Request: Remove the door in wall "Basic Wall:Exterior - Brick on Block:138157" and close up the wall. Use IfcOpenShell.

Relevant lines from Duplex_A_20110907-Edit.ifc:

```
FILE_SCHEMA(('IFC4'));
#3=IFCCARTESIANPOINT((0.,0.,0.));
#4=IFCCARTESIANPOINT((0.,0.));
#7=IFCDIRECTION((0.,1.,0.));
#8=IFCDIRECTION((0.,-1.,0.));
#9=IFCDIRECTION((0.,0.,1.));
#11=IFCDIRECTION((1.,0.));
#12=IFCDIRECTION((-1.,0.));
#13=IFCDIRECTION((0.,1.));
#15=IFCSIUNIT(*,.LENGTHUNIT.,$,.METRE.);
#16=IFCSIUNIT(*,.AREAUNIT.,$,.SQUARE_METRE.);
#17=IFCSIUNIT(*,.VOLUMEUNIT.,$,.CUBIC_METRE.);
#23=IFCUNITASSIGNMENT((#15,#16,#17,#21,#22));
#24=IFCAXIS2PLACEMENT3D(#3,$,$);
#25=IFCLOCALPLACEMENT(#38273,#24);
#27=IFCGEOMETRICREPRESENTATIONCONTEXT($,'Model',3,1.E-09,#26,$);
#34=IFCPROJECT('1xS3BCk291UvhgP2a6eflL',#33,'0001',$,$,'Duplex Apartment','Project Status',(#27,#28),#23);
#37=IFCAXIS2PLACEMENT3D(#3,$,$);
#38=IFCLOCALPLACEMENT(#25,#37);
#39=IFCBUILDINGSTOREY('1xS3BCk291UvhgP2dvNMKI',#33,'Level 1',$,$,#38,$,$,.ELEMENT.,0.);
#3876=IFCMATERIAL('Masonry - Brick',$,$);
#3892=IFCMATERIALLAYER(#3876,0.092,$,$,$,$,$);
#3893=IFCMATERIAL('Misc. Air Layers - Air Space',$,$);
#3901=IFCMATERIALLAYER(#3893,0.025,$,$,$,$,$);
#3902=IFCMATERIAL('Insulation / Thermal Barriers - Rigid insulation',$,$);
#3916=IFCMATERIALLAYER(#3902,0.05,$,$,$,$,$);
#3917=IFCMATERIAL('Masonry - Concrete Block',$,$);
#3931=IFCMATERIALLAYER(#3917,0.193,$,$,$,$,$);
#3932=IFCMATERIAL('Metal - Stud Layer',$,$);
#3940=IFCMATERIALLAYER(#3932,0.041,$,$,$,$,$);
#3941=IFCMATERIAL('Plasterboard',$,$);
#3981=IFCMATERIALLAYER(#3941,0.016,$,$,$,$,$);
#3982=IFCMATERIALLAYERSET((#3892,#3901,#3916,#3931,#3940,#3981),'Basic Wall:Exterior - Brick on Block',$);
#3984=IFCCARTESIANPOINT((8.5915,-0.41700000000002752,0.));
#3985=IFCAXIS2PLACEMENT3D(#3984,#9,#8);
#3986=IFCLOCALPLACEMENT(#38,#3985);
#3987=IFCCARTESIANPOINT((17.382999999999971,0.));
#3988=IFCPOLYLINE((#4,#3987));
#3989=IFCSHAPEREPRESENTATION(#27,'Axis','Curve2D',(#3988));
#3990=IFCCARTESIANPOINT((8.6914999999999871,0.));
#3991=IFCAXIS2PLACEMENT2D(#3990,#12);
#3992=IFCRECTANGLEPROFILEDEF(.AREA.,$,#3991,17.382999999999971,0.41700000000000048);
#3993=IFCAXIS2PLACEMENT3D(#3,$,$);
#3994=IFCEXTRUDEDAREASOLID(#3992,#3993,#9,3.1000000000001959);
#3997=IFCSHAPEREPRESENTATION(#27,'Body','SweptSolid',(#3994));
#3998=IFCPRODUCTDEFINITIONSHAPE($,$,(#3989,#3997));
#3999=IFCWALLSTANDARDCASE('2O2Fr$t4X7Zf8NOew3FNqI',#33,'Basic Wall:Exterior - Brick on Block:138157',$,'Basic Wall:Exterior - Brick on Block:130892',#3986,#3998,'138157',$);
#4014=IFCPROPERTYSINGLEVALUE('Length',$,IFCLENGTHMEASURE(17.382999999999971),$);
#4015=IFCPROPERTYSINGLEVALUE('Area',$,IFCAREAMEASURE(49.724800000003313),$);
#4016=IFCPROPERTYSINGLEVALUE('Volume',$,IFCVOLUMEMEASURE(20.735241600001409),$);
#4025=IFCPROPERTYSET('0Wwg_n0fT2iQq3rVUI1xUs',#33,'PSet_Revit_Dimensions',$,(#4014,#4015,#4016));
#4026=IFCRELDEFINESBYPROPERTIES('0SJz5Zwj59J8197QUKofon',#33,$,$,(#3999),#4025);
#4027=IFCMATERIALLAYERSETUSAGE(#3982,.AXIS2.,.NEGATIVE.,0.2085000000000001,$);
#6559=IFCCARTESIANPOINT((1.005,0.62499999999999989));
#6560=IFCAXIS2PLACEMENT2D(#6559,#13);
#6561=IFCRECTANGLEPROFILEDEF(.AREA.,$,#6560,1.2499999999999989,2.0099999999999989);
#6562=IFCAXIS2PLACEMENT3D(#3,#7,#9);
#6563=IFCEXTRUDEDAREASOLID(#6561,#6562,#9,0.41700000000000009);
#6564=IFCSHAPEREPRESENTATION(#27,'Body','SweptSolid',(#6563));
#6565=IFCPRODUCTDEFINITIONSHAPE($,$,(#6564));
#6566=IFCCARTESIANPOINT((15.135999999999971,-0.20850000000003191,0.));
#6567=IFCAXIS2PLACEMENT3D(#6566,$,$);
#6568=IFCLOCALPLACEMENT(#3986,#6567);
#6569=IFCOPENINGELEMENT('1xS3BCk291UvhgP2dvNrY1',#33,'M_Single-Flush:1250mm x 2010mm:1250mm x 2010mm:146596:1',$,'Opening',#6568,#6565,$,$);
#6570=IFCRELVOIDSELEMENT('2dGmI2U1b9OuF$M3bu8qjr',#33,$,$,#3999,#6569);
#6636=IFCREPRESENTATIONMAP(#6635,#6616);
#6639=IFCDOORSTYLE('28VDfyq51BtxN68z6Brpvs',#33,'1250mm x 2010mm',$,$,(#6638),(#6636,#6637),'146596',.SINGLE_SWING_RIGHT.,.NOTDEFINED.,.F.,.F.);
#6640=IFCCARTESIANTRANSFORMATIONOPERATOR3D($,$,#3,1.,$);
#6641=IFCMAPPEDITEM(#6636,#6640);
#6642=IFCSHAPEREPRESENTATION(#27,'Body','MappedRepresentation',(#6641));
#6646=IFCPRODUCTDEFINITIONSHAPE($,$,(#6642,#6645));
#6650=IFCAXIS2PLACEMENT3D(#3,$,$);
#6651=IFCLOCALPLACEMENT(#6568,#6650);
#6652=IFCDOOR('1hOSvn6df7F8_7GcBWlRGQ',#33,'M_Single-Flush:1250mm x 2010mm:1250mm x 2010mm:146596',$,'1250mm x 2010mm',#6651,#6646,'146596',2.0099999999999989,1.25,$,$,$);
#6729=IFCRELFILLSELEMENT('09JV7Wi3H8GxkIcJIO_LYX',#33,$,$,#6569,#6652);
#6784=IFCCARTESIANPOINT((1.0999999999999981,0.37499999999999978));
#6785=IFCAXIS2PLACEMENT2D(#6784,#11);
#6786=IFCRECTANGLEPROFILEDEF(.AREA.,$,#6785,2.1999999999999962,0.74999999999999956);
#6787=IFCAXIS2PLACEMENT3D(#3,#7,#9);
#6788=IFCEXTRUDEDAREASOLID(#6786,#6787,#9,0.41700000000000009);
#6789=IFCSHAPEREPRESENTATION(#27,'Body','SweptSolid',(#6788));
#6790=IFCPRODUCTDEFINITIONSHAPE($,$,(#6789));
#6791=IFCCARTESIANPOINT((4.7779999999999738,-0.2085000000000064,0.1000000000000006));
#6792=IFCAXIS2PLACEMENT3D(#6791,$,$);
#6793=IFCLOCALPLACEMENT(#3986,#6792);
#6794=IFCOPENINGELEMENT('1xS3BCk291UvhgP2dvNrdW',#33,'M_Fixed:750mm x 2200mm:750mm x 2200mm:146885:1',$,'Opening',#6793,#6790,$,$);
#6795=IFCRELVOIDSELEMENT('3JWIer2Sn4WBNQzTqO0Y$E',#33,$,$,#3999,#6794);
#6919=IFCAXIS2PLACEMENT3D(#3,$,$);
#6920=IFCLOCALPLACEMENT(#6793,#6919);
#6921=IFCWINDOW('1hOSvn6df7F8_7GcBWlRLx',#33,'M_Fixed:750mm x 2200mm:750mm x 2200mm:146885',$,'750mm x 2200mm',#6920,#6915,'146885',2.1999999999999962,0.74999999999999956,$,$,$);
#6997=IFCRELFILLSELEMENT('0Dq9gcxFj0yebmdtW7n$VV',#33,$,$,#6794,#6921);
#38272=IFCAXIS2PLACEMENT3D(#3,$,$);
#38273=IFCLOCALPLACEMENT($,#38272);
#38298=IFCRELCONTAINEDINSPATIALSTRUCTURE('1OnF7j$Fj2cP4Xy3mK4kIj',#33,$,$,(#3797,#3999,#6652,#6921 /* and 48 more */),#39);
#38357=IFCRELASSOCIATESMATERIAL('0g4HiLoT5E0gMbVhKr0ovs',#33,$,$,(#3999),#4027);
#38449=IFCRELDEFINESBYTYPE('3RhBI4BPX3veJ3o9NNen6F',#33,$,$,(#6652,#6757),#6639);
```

```python
import ifcopenshell
import ifcopenshell.api.feature
import ifcopenshell.api.pset
import ifcopenshell.api.root
import ifcopenshell.geom
import ifcopenshell.util.element
import ifcopenshell.util.shape
import ifcopenshell.util.unit

model = ifcopenshell.open("Duplex_A_20110907-Edit.ifc")
area_scale = ifcopenshell.util.unit.calculate_unit_scale(model, "AREAUNIT")
volume_scale = ifcopenshell.util.unit.calculate_unit_scale(model, "VOLUMEUNIT")
settings = ifcopenshell.geom.settings()


def volume(element):
    """Net volume in cubic metres, openings subtracted."""
    shape = ifcopenshell.geom.create_shape(settings, element)
    return ifcopenshell.util.shape.get_volume(shape.geometry)


door = model.by_guid("1hOSvn6df7F8_7GcBWlRGQ")
opening = door.FillsVoids[0].RelatingOpeningElement
wall = opening.VoidsElements[0].RelatingBuildingElement
before = volume(wall)

ifcopenshell.api.root.remove_product(model, product=door)
ifcopenshell.api.feature.remove_feature(model, feature=opening)

after = volume(wall)
thickness = 0.417  # wall thickness in metres

# Update the wall's stored quantities.
pset = model.by_id(ifcopenshell.util.element.get_pset(wall, "PSet_Revit_Dimensions", should_inherit=False)["id"])
ifcopenshell.api.pset.edit_pset(model, pset=pset, properties={
    "Area": model.create_entity("IfcAreaMeasure", after / thickness / area_scale),
    "Volume": model.create_entity("IfcVolumeMeasure", after / volume_scale),
})

print(f"wall volume {before:.3f} -> {after:.3f} m3")

model.write("Duplex_A_20110907-Edit-out.ifc")
```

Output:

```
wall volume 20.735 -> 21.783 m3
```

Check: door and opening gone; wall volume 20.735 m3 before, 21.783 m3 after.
